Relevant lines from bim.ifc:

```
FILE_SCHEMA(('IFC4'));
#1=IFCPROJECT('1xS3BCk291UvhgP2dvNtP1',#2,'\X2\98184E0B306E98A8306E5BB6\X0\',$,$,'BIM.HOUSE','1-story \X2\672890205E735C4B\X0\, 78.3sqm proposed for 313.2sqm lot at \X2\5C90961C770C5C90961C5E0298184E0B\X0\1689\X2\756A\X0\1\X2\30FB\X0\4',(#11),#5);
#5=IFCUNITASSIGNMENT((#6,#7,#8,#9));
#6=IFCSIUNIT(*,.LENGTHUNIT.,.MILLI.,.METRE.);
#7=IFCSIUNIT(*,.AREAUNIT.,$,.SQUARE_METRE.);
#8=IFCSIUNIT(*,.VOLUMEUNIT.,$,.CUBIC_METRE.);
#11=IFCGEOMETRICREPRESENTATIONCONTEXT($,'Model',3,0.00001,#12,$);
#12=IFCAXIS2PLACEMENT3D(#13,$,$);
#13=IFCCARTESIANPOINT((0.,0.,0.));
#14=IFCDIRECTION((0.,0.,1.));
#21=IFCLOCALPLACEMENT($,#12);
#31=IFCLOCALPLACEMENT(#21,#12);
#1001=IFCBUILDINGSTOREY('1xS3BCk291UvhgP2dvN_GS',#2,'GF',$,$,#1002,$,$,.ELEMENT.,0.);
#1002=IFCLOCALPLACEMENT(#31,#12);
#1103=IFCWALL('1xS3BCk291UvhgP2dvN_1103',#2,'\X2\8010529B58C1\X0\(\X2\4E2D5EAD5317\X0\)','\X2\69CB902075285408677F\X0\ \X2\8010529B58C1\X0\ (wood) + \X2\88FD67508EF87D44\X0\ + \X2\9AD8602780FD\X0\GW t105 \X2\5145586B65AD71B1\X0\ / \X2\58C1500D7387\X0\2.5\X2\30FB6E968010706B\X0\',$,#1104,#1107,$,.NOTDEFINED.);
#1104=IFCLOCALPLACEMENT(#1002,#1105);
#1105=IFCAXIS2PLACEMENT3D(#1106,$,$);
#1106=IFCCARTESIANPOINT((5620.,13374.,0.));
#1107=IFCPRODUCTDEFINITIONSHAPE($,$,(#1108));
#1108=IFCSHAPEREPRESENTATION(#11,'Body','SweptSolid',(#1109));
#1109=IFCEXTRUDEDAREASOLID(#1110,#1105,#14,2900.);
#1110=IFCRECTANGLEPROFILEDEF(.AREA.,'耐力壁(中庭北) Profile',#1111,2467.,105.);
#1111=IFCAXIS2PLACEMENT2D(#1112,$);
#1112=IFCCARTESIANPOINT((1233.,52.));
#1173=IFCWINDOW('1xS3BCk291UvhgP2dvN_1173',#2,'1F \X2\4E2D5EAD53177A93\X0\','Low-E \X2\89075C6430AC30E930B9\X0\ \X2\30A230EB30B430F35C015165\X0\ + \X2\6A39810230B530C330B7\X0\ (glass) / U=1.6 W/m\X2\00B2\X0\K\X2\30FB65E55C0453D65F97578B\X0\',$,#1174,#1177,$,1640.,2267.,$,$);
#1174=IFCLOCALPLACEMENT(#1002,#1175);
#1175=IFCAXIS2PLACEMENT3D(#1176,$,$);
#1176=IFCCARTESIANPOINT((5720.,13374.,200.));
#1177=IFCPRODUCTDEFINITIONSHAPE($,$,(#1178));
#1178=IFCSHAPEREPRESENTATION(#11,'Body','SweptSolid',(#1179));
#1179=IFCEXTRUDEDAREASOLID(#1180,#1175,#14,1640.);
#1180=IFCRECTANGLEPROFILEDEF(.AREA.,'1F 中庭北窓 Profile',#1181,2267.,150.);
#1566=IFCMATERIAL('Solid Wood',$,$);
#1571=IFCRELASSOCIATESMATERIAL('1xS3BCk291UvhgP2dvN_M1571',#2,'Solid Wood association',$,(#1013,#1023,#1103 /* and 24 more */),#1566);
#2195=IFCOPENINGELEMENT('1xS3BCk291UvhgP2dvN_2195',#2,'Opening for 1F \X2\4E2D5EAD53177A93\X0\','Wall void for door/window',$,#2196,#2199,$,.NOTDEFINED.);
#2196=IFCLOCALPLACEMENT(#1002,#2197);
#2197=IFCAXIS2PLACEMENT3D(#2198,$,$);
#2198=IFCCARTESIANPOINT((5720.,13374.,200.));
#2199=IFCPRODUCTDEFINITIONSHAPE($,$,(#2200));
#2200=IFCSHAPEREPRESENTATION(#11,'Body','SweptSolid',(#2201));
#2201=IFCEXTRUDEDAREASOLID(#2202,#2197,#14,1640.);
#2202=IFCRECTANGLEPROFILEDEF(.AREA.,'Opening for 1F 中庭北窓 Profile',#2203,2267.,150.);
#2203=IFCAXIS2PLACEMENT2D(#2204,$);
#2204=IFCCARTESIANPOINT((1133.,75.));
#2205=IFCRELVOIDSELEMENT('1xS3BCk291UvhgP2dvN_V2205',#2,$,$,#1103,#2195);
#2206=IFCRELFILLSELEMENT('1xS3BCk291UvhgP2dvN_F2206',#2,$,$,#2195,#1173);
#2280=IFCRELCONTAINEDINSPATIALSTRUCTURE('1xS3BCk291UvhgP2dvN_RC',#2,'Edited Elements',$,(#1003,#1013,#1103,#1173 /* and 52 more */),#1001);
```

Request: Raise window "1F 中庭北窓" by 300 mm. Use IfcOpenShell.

```python
import numpy as np
import ifcopenshell
import ifcopenshell.api.geometry
import ifcopenshell.util.placement
import ifcopenshell.util.unit

model = ifcopenshell.open("bim.ifc")
unit_scale = ifcopenshell.util.unit.calculate_unit_scale(model)

window = model.by_guid("1xS3BCk291UvhgP2dvN_1173")
opening = window.FillsVoids[0].RelatingOpeningElement
dz = 0.3 / unit_scale

shift = np.array([0.0, 0.0, dz])
# The window is not placed relative to its opening, so move both.
for product in (opening, window):
    matrix = ifcopenshell.util.placement.get_local_placement(product.ObjectPlacement)
    matrix[:3, 3] += shift
    ifcopenshell.api.geometry.edit_object_placement(model, product=product, matrix=matrix, is_si=False)

print(f"moved by {dz * unit_scale:+.3f} m")

model.write("bim-out.ifc")
```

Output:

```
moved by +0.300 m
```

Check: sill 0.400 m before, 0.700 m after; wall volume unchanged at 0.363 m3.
